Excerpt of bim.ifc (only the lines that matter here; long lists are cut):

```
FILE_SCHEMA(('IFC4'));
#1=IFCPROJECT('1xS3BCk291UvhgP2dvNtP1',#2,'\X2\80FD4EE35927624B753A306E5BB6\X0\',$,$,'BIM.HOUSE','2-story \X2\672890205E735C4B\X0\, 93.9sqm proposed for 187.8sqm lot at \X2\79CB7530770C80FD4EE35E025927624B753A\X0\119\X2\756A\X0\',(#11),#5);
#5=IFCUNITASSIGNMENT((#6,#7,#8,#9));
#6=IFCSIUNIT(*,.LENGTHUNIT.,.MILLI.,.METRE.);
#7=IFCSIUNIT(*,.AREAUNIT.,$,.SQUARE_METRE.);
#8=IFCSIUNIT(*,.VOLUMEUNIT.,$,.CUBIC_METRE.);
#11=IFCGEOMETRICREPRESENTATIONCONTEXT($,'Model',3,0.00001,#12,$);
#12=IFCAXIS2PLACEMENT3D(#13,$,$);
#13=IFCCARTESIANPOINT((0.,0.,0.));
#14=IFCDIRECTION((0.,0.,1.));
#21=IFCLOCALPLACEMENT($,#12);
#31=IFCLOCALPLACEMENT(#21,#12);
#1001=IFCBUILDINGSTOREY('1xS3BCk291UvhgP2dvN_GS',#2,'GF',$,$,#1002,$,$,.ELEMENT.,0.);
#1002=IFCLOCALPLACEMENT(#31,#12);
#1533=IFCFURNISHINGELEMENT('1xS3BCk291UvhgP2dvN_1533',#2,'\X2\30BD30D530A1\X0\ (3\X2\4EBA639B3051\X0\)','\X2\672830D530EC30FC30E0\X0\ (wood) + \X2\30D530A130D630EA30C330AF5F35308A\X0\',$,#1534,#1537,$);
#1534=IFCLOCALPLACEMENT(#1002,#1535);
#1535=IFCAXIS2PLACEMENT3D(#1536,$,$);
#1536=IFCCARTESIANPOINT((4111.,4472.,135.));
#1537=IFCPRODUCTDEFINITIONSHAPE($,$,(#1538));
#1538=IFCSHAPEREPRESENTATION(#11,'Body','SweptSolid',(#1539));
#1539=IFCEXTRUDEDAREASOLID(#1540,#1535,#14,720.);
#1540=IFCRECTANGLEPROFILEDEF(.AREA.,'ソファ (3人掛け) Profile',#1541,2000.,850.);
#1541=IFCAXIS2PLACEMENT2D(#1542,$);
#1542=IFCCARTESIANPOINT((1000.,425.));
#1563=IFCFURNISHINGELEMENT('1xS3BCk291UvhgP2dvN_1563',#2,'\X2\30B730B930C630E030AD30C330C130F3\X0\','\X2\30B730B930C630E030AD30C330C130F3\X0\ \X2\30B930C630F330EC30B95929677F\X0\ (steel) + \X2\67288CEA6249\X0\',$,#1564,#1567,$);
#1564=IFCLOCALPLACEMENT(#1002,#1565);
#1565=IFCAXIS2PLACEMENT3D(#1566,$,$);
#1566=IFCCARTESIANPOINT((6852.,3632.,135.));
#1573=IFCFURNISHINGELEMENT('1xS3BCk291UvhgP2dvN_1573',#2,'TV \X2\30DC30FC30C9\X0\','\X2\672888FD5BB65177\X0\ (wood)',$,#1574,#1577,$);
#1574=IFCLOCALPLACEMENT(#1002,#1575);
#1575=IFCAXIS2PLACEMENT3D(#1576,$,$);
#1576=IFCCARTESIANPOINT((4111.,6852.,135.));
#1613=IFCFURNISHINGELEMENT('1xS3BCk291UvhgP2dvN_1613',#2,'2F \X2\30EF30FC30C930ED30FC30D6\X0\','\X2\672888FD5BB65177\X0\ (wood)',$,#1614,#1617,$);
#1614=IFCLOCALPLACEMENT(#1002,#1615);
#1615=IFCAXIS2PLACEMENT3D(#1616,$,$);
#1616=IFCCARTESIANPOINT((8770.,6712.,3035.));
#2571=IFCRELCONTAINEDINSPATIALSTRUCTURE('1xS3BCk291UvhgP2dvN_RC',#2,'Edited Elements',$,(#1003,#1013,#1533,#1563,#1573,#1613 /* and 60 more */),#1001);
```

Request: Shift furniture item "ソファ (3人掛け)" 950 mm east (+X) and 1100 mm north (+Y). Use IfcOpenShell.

```python
import ifcopenshell
import ifcopenshell.api.geometry
import ifcopenshell.util.placement
import ifcopenshell.util.unit

model = ifcopenshell.open("bim.ifc")
unit_scale = ifcopenshell.util.unit.calculate_unit_scale(model)

item = model.by_guid("1xS3BCk291UvhgP2dvN_1533")
matrix = ifcopenshell.util.placement.get_local_placement(item.ObjectPlacement)
matrix[0, 3] += 0.95 / unit_scale
matrix[1, 3] += 1.1 / unit_scale
ifcopenshell.api.geometry.edit_object_placement(model, product=item, matrix=matrix, is_si=False)

print(ifcopenshell.util.placement.get_local_placement(item.ObjectPlacement).round(3) + 0.0)

model.write("bim_v2.ifc")
```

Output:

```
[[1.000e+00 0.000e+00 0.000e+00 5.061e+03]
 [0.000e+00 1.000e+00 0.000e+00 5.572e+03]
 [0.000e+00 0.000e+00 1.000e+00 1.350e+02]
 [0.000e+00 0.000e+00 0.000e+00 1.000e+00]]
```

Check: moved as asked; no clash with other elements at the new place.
